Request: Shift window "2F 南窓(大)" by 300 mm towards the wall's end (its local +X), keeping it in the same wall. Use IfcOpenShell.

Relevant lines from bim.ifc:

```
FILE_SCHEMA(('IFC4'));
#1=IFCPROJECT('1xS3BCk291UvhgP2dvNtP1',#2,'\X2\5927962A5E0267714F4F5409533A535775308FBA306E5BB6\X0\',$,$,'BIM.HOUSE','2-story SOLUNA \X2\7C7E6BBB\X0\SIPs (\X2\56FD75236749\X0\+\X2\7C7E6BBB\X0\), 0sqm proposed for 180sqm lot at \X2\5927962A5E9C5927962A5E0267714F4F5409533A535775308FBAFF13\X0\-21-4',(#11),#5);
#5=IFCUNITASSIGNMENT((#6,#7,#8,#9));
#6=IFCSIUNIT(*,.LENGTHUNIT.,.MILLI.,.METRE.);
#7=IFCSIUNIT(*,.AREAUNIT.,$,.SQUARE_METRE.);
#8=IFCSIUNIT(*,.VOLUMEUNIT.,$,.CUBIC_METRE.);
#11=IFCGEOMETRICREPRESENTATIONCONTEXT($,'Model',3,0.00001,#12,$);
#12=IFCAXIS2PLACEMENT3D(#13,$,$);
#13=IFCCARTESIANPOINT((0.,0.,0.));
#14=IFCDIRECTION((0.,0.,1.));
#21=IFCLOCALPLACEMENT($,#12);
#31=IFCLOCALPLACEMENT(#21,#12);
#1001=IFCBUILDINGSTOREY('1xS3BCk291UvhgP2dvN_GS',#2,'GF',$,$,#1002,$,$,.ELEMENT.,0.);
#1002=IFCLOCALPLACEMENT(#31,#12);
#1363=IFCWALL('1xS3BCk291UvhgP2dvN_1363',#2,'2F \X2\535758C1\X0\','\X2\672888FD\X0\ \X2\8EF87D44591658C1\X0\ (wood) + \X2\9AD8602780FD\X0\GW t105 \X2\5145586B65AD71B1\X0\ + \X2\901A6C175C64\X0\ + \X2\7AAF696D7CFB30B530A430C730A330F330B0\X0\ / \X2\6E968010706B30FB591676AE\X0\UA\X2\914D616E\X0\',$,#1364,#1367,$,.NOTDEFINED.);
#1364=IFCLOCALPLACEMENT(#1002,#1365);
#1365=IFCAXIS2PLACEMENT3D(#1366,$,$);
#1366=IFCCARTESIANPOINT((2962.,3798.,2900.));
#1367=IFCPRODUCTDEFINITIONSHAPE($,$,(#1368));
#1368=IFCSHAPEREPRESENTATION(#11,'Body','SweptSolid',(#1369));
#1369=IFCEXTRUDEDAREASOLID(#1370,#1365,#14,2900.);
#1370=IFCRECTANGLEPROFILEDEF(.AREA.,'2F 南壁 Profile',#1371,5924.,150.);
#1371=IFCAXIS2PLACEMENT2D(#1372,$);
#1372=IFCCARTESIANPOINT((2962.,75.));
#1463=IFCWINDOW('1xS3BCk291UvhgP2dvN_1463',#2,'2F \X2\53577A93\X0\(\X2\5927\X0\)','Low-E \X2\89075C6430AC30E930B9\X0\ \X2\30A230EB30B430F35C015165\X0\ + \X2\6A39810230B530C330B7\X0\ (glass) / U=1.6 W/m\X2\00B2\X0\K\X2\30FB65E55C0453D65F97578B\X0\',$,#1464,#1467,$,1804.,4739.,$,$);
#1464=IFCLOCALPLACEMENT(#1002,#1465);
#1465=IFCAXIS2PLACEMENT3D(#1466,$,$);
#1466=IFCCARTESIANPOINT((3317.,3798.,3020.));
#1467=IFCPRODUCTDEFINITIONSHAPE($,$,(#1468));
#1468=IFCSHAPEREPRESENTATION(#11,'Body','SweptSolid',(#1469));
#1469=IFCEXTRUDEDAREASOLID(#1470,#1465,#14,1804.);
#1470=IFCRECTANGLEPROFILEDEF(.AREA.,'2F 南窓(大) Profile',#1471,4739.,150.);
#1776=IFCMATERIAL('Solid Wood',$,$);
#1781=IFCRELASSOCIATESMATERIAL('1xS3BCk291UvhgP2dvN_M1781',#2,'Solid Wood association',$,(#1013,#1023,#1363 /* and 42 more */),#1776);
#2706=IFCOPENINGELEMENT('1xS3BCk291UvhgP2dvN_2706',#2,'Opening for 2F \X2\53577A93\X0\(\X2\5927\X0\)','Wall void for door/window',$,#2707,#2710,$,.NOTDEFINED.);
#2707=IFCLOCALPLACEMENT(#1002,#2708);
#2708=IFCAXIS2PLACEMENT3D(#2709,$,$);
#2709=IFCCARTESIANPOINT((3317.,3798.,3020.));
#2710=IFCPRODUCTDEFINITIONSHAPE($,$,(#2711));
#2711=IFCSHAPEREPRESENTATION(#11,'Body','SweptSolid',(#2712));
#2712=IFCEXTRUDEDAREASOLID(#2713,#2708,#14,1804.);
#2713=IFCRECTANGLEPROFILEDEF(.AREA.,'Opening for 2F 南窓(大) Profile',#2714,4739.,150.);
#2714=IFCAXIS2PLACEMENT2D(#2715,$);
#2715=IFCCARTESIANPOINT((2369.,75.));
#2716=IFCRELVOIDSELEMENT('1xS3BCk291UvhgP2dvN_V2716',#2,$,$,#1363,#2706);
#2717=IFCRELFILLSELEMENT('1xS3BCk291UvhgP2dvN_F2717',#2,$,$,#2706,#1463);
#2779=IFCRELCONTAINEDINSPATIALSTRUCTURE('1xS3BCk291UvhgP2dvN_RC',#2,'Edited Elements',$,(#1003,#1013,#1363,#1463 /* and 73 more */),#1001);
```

```python
import ifcopenshell
import ifcopenshell.api.geometry
import ifcopenshell.util.placement
import ifcopenshell.util.unit

model = ifcopenshell.open("bim.ifc")
unit_scale = ifcopenshell.util.unit.calculate_unit_scale(model)

window = model.by_guid("1xS3BCk291UvhgP2dvN_1463")
opening = window.FillsVoids[0].RelatingOpeningElement
wall = opening.VoidsElements[0].RelatingBuildingElement

wall_matrix = ifcopenshell.util.placement.get_local_placement(wall.ObjectPlacement)
shift = wall_matrix[:3, 0] * 0.3 / unit_scale
before = ifcopenshell.util.placement.get_local_placement(window.ObjectPlacement)[:3, 3].copy()

# The window is not placed relative to its opening, so move both.
for product in (opening, window):
    matrix = ifcopenshell.util.placement.get_local_placement(product.ObjectPlacement)
    matrix[:3, 3] += shift
    ifcopenshell.api.geometry.edit_object_placement(model, product=product, matrix=matrix, is_si=False)

after = ifcopenshell.util.placement.get_local_placement(window.ObjectPlacement)[:3, 3]
print("window moved by", (after - before).round(3) + 0.0)

model.write("bim-out.ifc")
```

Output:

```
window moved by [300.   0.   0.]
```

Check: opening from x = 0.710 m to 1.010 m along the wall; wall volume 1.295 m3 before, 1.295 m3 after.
